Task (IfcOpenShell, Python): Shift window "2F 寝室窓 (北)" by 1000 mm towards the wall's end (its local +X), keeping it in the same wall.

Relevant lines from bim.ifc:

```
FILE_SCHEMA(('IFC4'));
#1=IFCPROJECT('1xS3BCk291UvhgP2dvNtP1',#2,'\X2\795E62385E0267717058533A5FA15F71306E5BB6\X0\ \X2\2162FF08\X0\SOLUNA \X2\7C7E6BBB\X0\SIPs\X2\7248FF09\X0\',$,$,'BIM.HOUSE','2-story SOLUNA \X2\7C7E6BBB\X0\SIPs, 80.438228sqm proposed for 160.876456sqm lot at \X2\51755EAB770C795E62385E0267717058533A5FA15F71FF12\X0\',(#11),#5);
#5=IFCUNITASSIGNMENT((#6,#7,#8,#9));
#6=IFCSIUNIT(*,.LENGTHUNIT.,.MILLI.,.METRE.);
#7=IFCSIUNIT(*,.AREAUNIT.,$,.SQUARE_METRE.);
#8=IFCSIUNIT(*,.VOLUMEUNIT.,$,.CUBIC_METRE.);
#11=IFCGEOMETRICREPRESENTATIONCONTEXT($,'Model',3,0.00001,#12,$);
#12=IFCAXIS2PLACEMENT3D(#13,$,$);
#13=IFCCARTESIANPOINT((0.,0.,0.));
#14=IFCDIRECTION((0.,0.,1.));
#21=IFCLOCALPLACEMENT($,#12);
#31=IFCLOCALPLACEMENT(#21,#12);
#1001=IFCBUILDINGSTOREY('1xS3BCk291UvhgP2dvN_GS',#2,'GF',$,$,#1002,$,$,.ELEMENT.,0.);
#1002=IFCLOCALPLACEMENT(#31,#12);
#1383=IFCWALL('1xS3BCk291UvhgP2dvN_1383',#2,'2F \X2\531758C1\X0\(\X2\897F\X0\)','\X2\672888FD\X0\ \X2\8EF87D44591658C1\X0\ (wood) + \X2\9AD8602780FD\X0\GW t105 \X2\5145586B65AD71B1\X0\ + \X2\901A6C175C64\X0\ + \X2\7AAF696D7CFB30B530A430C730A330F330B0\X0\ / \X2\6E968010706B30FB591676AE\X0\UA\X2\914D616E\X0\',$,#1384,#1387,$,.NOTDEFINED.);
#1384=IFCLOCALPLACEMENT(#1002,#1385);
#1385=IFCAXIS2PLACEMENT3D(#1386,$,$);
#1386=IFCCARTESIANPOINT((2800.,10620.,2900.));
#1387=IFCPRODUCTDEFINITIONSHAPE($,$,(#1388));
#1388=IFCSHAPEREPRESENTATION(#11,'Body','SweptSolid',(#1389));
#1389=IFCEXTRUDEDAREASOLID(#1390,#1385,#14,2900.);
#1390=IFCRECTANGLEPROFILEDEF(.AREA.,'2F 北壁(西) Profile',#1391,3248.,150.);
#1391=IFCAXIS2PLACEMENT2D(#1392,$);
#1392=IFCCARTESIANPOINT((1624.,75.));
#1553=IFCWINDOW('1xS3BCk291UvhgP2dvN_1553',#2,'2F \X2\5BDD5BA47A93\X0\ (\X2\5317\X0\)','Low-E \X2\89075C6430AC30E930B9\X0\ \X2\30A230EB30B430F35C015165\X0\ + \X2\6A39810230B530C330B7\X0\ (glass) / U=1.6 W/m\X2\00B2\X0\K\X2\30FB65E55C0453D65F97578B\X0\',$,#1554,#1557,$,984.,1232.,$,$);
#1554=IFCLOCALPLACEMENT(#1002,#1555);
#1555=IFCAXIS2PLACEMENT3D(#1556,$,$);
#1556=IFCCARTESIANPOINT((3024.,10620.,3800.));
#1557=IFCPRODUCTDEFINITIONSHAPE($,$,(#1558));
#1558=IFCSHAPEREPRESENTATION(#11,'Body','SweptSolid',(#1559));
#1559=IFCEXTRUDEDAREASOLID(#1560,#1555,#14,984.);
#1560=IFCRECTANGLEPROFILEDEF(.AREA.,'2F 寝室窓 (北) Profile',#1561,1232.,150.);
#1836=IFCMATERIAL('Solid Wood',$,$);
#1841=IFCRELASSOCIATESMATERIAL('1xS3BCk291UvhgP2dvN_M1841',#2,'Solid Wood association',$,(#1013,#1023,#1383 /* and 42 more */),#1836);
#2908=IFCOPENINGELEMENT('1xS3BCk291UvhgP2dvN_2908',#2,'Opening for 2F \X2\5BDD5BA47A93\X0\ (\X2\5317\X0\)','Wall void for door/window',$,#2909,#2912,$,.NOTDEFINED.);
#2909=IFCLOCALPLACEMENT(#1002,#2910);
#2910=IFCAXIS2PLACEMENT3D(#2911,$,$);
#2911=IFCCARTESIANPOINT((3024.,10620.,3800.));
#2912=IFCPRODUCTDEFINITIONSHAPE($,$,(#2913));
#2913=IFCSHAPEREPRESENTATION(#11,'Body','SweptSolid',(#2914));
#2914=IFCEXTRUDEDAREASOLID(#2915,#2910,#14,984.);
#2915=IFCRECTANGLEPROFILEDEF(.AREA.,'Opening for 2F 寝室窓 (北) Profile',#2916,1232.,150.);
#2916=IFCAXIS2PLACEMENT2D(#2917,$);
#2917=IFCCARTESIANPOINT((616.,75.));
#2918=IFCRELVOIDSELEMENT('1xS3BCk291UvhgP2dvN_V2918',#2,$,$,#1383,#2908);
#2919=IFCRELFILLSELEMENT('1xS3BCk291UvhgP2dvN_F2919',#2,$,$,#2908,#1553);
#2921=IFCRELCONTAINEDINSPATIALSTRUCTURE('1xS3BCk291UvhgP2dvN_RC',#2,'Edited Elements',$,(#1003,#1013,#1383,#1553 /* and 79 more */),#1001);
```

```python
import ifcopenshell
import ifcopenshell.api.geometry
import ifcopenshell.util.placement
import ifcopenshell.util.unit

model = ifcopenshell.open("bim.ifc")
unit_scale = ifcopenshell.util.unit.calculate_unit_scale(model)

window = model.by_id(1553)
opening = window.FillsVoids[0].RelatingOpeningElement
wall = opening.VoidsElements[0].RelatingBuildingElement

wall_matrix = ifcopenshell.util.placement.get_local_placement(wall.ObjectPlacement)
shift = wall_matrix[:3, 0] * 1 / unit_scale
before = ifcopenshell.util.placement.get_local_placement(window.ObjectPlacement)[:3, 3].copy()

# The window is not placed relative to its opening, so move both.
for product in (opening, window):
    matrix = ifcopenshell.util.placement.get_local_placement(product.ObjectPlacement)
    matrix[:3, 3] += shift
    ifcopenshell.api.geometry.edit_object_placement(model, product=product, matrix=matrix, is_si=False)

after = ifcopenshell.util.placement.get_local_placement(window.ObjectPlacement)[:3, 3]
print("window moved by", (after - before).round(3) + 0.0)

model.write("bim_v2.ifc")
```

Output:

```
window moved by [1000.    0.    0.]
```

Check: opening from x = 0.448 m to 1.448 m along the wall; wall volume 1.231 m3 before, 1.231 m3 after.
